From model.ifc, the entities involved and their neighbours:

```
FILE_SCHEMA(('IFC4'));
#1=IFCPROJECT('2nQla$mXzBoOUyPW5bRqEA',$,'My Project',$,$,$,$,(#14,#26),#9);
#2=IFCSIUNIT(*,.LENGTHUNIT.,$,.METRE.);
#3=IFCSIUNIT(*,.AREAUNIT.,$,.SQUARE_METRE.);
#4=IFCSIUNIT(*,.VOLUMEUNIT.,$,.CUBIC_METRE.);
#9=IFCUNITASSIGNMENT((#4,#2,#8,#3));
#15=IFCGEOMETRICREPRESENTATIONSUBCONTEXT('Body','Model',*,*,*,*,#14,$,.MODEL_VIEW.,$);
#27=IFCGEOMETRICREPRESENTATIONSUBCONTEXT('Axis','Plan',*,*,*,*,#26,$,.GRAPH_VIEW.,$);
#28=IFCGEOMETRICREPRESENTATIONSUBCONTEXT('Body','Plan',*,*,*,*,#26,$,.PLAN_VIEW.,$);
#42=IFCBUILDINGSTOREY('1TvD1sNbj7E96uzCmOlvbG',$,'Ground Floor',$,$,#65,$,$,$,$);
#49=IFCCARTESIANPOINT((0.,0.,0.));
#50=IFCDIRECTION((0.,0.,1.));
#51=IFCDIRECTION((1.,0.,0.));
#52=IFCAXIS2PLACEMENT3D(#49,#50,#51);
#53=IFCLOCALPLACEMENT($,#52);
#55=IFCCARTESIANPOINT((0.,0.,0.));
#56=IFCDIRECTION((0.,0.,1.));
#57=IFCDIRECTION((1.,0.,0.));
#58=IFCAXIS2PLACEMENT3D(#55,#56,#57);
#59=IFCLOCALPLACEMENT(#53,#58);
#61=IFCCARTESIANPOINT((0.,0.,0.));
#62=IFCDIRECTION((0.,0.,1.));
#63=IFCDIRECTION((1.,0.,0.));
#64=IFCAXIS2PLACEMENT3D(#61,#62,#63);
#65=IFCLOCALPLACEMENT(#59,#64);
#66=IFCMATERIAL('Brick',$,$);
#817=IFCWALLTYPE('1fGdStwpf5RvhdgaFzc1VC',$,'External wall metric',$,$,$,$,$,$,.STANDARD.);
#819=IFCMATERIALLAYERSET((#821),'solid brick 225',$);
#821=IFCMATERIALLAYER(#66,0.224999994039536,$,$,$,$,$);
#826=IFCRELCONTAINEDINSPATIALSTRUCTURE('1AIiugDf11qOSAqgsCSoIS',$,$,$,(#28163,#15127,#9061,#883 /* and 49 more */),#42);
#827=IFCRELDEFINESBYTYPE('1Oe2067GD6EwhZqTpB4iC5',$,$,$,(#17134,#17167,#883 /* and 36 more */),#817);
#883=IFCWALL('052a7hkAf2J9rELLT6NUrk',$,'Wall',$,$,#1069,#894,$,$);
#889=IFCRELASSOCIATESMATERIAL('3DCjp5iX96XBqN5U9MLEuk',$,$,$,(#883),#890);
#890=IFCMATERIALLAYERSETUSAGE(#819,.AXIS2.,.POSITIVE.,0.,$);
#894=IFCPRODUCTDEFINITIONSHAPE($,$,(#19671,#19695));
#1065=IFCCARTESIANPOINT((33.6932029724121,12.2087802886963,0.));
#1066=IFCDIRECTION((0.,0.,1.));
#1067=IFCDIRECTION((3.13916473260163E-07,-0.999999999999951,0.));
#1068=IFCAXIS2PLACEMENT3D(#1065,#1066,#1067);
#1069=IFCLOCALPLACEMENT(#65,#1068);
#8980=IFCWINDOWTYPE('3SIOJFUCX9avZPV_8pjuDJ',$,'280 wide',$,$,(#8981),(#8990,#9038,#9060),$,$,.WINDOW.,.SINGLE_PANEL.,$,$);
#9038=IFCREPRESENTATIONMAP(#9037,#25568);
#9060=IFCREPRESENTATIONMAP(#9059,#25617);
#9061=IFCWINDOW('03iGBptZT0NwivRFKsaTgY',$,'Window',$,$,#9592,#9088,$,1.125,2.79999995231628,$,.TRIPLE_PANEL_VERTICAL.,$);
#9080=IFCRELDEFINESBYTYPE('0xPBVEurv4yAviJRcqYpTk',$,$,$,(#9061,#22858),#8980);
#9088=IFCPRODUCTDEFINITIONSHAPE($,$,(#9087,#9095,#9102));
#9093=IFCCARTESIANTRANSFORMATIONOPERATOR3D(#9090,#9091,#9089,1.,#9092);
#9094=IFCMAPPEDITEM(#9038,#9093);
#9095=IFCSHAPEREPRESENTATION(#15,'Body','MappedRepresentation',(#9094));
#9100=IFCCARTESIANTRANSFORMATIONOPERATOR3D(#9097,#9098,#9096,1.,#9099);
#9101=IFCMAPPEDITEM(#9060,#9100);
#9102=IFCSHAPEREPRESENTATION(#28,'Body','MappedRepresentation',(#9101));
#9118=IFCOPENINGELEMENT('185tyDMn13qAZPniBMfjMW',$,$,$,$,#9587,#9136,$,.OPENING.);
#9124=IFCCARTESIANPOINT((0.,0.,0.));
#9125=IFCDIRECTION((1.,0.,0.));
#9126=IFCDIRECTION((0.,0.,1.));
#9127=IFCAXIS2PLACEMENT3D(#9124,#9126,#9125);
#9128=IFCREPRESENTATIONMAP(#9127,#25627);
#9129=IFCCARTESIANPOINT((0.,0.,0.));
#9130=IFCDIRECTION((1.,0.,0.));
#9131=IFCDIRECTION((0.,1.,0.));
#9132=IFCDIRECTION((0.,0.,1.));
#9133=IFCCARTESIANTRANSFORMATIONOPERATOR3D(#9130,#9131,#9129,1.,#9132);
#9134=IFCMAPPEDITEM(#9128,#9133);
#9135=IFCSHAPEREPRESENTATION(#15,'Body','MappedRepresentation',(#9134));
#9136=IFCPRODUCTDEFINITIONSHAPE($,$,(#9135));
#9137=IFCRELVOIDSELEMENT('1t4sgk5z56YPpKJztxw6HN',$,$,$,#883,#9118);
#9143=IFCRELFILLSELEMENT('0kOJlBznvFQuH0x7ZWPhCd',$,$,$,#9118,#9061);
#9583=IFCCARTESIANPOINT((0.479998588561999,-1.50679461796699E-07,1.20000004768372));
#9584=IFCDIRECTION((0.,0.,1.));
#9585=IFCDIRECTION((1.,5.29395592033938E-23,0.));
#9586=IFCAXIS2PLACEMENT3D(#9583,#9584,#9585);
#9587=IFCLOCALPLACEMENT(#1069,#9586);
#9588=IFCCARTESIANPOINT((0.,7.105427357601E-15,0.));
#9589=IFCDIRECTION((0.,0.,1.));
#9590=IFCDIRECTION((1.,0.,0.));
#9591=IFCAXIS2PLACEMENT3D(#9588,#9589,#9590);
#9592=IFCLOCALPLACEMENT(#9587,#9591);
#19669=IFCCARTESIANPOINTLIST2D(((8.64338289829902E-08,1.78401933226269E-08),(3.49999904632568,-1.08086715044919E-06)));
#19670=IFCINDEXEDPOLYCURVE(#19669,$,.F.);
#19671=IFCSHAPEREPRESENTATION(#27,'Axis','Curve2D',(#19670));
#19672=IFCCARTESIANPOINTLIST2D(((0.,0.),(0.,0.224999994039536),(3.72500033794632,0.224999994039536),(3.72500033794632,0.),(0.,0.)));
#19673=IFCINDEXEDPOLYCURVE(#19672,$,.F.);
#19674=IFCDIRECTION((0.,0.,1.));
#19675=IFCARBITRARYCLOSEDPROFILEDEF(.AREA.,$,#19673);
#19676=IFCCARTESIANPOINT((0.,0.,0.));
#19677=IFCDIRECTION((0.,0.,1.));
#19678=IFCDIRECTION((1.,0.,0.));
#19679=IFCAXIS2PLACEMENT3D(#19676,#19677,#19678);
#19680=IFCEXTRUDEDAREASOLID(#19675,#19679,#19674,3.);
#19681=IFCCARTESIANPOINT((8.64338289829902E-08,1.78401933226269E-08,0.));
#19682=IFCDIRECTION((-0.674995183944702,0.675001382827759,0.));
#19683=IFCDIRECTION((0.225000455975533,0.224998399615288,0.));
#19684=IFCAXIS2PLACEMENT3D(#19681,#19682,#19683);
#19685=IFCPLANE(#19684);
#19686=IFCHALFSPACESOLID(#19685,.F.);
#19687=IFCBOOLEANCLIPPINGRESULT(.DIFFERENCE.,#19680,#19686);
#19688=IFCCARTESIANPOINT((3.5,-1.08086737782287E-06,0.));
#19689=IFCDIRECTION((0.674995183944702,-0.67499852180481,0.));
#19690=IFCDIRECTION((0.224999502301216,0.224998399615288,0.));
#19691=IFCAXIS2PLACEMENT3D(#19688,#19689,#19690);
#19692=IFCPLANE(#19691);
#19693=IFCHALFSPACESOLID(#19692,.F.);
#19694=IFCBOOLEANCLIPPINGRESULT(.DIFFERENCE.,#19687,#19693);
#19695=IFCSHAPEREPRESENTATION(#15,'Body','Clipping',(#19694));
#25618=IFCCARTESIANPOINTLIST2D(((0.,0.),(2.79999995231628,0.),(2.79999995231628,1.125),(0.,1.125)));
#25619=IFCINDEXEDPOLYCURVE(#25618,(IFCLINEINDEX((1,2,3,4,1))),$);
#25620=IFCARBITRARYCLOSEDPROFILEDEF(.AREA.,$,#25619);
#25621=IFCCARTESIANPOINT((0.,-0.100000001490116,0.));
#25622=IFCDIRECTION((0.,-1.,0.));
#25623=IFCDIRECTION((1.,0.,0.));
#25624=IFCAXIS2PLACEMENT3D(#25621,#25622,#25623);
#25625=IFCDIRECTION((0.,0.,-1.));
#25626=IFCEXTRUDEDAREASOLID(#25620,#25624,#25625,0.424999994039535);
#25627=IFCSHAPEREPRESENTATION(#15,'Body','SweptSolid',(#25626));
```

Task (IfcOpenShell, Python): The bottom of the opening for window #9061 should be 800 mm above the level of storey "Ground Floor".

```python
import numpy as np
import ifcopenshell
import ifcopenshell.api.geometry
import ifcopenshell.geom
import ifcopenshell.util.element
import ifcopenshell.util.placement
import ifcopenshell.util.shape
import ifcopenshell.util.unit

model = ifcopenshell.open("model.ifc")
unit_scale = ifcopenshell.util.unit.calculate_unit_scale(model)

window = model.by_guid("03iGBptZT0NwivRFKsaTgY")
opening = window.FillsVoids[0].RelatingOpeningElement
storey = ifcopenshell.util.element.get_container(window, ifc_class="IfcBuildingStorey")
level = ifcopenshell.util.placement.get_local_placement(storey.ObjectPlacement)[2, 3]

# The opening's origin need not be at the sill, so measure its lowest point.
shape = ifcopenshell.geom.create_shape(ifcopenshell.geom.settings(), opening)
bottom = ifcopenshell.util.shape.get_shape_bottom_elevation(shape, shape.geometry) / unit_scale
dz = level + 0.8 / unit_scale - bottom

shift = np.array([0.0, 0.0, dz])
# The window is placed relative to its opening, so it follows when the opening moves.
matrix = ifcopenshell.util.placement.get_local_placement(opening.ObjectPlacement)
matrix[:3, 3] += shift
ifcopenshell.api.geometry.edit_object_placement(
    model, product=opening, matrix=matrix, is_si=False, should_transform_children=True
)

print(f"moved by {dz * unit_scale:+.3f} m")

model.write("model_edited.ifc")
```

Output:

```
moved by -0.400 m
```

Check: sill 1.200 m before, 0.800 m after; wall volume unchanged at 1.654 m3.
